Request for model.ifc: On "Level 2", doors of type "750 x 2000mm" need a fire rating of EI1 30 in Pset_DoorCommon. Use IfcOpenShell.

First a look at what the model holds.

```python
import ifcopenshell
import ifcopenshell.util.element

model = ifcopenshell.open("model.ifc")
print(model.schema)
storey = next(s for s in model.by_type("IfcBuildingStorey") if s.Name == "Level 2")
doors = [e for e in ifcopenshell.util.element.get_decomposition(storey) if e.is_a("IfcDoor")]
seen = {}
for e in doors:
    element_type = ifcopenshell.util.element.get_type(e)
    key = (element_type.Name if element_type != e and element_type else None, ifcopenshell.util.element.get_pset(e, "Pset_DoorCommon", "FireRating"))
    seen[key] = seen.get(key, 0) + 1
for (name, value), count in sorted(seen.items(), key=str):
    print(count, "x", name, "|", value)
```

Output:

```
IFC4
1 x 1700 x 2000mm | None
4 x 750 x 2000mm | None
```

```python
import ifcopenshell
import ifcopenshell.api.pset
import ifcopenshell.util.element

model = ifcopenshell.open("model.ifc")

storey = next(s for s in model.by_type("IfcBuildingStorey") if s.Name == "Level 2")
doors = [e for e in ifcopenshell.util.element.get_decomposition(storey) if e.is_a("IfcDoor")]

count = 0
for e in doors:
    element_type = ifcopenshell.util.element.get_type(e)
    if element_type in (None, e) or element_type.Name != "750 x 2000mm":
        continue
    # add_pset returns the element's existing set when there is one.
    pset = ifcopenshell.api.pset.add_pset(model, product=e, name="Pset_DoorCommon")
    ifcopenshell.api.pset.edit_pset(model, pset=pset, properties={"FireRating": "EI1 30"})
    count += 1

print(count, "doors updated")

model.write("model_edited.ifc")
```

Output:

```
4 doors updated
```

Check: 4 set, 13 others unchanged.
